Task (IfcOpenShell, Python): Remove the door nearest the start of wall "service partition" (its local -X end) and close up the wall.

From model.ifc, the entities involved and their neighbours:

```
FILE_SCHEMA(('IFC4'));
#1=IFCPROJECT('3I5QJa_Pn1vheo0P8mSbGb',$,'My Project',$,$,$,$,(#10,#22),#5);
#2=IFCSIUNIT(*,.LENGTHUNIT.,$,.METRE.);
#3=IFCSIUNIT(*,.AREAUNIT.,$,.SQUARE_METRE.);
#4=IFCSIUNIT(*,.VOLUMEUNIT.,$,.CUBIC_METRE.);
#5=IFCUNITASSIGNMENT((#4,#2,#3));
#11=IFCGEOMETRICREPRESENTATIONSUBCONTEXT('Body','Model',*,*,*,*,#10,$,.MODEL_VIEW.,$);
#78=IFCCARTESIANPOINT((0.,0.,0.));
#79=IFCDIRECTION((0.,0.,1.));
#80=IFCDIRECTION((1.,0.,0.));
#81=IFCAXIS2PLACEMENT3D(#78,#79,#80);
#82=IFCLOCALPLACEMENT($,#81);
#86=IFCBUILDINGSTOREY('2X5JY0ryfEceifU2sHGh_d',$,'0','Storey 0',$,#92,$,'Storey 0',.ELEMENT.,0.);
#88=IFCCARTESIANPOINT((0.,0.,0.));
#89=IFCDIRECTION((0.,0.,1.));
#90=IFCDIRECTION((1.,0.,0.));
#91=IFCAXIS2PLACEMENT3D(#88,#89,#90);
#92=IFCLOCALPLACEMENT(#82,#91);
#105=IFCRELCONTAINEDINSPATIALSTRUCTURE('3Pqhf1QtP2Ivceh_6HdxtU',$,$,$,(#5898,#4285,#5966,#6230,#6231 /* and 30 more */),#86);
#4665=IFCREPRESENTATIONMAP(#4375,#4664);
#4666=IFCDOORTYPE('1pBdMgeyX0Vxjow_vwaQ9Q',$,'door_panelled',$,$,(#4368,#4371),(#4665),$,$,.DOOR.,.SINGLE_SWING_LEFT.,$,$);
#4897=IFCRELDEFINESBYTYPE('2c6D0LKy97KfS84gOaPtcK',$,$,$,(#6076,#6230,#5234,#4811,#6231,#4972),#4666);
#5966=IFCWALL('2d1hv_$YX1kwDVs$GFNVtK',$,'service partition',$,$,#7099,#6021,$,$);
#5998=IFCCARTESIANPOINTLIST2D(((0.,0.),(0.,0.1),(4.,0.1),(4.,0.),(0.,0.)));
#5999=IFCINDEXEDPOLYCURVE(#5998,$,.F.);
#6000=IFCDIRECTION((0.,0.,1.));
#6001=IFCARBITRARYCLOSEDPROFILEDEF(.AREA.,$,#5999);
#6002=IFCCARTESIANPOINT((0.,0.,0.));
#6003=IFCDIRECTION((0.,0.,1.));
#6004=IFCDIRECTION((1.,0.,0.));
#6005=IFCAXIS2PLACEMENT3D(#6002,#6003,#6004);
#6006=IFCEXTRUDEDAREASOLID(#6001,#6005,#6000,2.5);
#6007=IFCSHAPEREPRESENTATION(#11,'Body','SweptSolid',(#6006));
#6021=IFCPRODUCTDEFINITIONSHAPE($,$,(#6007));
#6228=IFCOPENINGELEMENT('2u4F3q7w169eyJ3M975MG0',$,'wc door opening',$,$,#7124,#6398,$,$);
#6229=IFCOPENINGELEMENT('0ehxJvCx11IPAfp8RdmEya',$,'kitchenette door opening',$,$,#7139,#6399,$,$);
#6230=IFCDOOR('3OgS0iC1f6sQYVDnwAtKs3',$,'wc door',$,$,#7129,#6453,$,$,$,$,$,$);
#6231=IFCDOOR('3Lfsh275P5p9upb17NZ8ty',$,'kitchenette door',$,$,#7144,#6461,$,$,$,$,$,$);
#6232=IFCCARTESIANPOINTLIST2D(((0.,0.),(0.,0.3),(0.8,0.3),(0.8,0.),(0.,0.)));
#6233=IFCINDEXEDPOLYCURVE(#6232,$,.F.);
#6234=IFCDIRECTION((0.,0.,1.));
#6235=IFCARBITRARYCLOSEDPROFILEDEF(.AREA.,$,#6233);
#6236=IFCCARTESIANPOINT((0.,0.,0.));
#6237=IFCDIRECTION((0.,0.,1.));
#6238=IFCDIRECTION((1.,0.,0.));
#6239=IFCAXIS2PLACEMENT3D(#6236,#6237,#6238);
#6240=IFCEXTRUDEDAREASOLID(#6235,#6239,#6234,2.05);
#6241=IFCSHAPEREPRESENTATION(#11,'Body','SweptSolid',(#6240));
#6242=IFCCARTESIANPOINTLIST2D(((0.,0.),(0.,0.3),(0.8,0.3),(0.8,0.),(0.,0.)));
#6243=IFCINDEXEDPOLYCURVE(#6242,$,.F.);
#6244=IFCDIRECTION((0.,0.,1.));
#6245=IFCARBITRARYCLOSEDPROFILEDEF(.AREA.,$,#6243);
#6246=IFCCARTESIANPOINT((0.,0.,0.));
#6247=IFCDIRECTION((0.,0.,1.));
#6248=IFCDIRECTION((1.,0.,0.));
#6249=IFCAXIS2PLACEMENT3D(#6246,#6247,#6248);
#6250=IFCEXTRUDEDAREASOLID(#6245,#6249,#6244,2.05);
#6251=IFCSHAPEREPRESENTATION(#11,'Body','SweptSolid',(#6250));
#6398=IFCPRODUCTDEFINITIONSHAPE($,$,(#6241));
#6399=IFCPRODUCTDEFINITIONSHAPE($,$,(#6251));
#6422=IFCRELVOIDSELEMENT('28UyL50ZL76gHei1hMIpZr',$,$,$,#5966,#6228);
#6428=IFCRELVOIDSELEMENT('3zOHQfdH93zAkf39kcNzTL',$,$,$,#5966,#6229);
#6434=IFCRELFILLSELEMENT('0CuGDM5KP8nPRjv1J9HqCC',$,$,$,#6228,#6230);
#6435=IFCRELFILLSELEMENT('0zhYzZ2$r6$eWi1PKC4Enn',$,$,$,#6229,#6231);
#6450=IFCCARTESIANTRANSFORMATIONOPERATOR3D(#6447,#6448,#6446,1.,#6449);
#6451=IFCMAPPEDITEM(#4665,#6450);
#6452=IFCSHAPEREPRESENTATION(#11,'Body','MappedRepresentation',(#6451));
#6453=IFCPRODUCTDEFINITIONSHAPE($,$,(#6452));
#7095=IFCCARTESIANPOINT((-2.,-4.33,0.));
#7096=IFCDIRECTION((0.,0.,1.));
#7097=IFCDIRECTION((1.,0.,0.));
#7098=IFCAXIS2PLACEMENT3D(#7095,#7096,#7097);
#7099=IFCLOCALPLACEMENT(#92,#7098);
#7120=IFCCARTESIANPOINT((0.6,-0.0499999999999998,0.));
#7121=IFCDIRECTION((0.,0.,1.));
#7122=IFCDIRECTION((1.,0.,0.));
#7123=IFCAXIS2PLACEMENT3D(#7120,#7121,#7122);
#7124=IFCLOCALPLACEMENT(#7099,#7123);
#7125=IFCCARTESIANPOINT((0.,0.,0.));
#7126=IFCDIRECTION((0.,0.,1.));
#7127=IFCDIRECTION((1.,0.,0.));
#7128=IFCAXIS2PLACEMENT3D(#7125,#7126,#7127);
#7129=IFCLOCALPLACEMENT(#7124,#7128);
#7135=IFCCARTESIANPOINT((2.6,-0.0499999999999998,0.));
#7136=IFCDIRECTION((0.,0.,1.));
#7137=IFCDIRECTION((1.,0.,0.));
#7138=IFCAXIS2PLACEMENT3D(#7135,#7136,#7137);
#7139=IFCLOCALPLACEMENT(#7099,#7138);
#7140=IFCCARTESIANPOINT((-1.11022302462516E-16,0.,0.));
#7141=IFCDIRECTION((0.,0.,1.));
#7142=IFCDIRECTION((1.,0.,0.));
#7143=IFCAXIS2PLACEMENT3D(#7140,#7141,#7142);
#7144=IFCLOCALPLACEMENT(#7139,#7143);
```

```python
import ifcopenshell
import ifcopenshell.api.feature
import ifcopenshell.api.root
import ifcopenshell.geom
import ifcopenshell.util.shape

model = ifcopenshell.open("model.ifc")
settings = ifcopenshell.geom.settings()


def volume(element):
    """Net volume in cubic metres, openings subtracted."""
    shape = ifcopenshell.geom.create_shape(settings, element)
    return ifcopenshell.util.shape.get_volume(shape.geometry)


door = model.by_guid("3OgS0iC1f6sQYVDnwAtKs3")
opening = door.FillsVoids[0].RelatingOpeningElement
wall = opening.VoidsElements[0].RelatingBuildingElement
before = volume(wall)

ifcopenshell.api.root.remove_product(model, product=door)
ifcopenshell.api.feature.remove_feature(model, feature=opening)

after = volume(wall)

print(f"wall volume {before:.3f} -> {after:.3f} m3")

model.write("model_updated.ifc")
```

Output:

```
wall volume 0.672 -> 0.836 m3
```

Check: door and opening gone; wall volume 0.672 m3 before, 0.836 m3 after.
